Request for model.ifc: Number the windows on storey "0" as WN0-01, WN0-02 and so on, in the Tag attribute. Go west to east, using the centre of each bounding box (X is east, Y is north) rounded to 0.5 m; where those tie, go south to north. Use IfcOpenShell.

First a look at what the model holds.

```python
import ifcopenshell
import ifcopenshell.util.element
import ifcopenshell.util.placement

model = ifcopenshell.open("model.ifc")
print(model.schema)
storey = next(s for s in model.by_type("IfcBuildingStorey") if s.Name == "0")
windows = [e for e in ifcopenshell.util.element.get_decomposition(storey) if e.is_a("IfcWindow")]
for e in sorted(windows, key=lambda e: e.id()):
    origin = ifcopenshell.util.placement.get_local_placement(e.ObjectPlacement)[:3, 3]
    print(e.id(), e.Tag, e.Name, origin.round(2) + 0.0, sep=" | ")
```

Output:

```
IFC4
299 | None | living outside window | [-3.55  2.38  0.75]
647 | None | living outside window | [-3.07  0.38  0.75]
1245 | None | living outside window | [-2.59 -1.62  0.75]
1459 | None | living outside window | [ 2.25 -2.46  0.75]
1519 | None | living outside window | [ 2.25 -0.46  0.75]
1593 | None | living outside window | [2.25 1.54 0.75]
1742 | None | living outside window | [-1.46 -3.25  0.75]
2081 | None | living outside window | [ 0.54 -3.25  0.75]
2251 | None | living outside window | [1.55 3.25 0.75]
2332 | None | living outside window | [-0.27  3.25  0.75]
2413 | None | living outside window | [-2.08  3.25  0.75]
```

```python
import ifcopenshell
import ifcopenshell.geom
import ifcopenshell.util.element
import ifcopenshell.util.shape

model = ifcopenshell.open("model.ifc")
settings = ifcopenshell.geom.settings()
settings.set("use-world-coords", True)


def centre(element):
    shape = ifcopenshell.geom.create_shape(settings, element)
    return ifcopenshell.util.shape.get_bbox_centroid(shape.geometry)


storey = next(s for s in model.by_type("IfcBuildingStorey") if s.Name == "0")
windows = [e for e in ifcopenshell.util.element.get_decomposition(storey) if e.is_a("IfcWindow")]

# Insertion points can sit at a corner or the storey origin, so sort by the geometry (in metres).
centres = {e: centre(e) for e in windows}
windows.sort(key=lambda e: (round(centres[e][0] / 0.5), centres[e][1]))

for i, e in enumerate(windows, start=1):
    number = f"WN0-{i:02d}"
    e.Tag = number
    print(e.id(), number)

model.write("model_v2.ifc")
```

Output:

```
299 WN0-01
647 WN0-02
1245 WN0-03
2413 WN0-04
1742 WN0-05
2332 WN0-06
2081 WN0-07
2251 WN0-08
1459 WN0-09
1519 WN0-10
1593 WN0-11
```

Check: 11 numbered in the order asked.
